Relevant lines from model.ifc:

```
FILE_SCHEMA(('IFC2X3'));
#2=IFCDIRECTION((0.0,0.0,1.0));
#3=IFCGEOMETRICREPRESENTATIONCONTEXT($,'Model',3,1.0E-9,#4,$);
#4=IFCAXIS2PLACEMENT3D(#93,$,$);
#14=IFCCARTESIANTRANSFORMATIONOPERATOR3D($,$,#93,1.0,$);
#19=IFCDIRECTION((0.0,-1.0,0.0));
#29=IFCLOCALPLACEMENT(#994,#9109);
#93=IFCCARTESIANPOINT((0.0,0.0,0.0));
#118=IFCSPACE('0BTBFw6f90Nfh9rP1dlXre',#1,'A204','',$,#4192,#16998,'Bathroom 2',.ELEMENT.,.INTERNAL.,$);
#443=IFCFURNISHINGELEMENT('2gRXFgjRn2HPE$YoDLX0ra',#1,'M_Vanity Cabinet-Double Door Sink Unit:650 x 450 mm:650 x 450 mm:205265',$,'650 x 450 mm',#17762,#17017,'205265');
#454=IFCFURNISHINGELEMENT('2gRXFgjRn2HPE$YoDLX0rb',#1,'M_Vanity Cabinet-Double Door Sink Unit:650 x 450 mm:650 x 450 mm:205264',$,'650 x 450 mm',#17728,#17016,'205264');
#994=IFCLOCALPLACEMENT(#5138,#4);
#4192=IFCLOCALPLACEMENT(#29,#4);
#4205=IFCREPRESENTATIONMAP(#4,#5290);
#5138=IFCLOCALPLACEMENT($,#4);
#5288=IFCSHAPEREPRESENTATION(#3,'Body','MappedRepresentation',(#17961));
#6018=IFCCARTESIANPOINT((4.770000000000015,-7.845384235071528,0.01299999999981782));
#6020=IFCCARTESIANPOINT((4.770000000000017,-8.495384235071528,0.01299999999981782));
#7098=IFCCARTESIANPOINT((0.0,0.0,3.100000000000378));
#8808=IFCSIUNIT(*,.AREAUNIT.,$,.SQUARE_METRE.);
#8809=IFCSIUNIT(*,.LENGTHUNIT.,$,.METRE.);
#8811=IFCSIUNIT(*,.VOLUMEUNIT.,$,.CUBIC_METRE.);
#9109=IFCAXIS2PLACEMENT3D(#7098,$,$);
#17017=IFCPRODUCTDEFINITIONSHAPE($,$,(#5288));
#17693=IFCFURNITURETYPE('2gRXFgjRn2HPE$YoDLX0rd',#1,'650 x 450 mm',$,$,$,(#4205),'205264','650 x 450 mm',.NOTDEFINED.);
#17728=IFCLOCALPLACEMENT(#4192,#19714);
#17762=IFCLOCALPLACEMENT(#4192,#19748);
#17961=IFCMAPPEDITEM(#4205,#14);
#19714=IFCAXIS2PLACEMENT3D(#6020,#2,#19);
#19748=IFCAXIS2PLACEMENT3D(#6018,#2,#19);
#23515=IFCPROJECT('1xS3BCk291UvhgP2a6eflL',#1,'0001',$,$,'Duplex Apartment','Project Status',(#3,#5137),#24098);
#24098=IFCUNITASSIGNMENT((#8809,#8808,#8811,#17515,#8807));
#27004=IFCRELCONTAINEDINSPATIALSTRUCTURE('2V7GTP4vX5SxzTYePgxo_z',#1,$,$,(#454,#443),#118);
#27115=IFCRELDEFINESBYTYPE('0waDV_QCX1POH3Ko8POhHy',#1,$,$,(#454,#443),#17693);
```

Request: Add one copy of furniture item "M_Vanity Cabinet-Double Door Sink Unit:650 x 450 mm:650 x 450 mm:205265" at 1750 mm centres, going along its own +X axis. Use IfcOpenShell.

```python
import ifcopenshell
import ifcopenshell.api.geometry
import ifcopenshell.api.root
import ifcopenshell.util.element
import ifcopenshell.util.placement

model = ifcopenshell.open("model.ifc")


def reuse_history(source, copy):
    """copy_class also copies each property set's owner history, people and application; keep the originals."""
    for rel in copy.IsDefinedBy:
        if rel.is_a("IfcRelDefinesByProperties") and (history := rel.RelatingPropertyDefinition.OwnerHistory):
            rel.RelatingPropertyDefinition.OwnerHistory = source.OwnerHistory
            ifcopenshell.util.element.remove_deep2(model, history)


source = model.by_guid("2gRXFgjRn2HPE$YoDLX0ra")
base = ifcopenshell.util.placement.get_local_placement(source.ObjectPlacement)
step = base[:3, 0] * 1.75

for i in range(1, 2):
    copy = ifcopenshell.api.root.copy_class(model, product=source)
    copy.Representation = ifcopenshell.util.element.copy_deep(
        model, source.Representation, exclude=["IfcGeometricRepresentationContext", "IfcRepresentationMap"]
    )
    copy.Name = "M_Vanity Cabinet-Double Door Sink Unit:650 x 450 mm:650 x 450 mm"
    copy.Tag = None
    reuse_history(source, copy)
    matrix = base.copy()
    matrix[:3, 3] += i * step
    print("added at", matrix[:3, 3].round(3) + 0.0)
    ifcopenshell.api.geometry.edit_object_placement(model, product=copy, matrix=matrix, is_si=False)

model.write("model-out.ifc")
```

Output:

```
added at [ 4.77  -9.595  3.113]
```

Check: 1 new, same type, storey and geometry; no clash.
